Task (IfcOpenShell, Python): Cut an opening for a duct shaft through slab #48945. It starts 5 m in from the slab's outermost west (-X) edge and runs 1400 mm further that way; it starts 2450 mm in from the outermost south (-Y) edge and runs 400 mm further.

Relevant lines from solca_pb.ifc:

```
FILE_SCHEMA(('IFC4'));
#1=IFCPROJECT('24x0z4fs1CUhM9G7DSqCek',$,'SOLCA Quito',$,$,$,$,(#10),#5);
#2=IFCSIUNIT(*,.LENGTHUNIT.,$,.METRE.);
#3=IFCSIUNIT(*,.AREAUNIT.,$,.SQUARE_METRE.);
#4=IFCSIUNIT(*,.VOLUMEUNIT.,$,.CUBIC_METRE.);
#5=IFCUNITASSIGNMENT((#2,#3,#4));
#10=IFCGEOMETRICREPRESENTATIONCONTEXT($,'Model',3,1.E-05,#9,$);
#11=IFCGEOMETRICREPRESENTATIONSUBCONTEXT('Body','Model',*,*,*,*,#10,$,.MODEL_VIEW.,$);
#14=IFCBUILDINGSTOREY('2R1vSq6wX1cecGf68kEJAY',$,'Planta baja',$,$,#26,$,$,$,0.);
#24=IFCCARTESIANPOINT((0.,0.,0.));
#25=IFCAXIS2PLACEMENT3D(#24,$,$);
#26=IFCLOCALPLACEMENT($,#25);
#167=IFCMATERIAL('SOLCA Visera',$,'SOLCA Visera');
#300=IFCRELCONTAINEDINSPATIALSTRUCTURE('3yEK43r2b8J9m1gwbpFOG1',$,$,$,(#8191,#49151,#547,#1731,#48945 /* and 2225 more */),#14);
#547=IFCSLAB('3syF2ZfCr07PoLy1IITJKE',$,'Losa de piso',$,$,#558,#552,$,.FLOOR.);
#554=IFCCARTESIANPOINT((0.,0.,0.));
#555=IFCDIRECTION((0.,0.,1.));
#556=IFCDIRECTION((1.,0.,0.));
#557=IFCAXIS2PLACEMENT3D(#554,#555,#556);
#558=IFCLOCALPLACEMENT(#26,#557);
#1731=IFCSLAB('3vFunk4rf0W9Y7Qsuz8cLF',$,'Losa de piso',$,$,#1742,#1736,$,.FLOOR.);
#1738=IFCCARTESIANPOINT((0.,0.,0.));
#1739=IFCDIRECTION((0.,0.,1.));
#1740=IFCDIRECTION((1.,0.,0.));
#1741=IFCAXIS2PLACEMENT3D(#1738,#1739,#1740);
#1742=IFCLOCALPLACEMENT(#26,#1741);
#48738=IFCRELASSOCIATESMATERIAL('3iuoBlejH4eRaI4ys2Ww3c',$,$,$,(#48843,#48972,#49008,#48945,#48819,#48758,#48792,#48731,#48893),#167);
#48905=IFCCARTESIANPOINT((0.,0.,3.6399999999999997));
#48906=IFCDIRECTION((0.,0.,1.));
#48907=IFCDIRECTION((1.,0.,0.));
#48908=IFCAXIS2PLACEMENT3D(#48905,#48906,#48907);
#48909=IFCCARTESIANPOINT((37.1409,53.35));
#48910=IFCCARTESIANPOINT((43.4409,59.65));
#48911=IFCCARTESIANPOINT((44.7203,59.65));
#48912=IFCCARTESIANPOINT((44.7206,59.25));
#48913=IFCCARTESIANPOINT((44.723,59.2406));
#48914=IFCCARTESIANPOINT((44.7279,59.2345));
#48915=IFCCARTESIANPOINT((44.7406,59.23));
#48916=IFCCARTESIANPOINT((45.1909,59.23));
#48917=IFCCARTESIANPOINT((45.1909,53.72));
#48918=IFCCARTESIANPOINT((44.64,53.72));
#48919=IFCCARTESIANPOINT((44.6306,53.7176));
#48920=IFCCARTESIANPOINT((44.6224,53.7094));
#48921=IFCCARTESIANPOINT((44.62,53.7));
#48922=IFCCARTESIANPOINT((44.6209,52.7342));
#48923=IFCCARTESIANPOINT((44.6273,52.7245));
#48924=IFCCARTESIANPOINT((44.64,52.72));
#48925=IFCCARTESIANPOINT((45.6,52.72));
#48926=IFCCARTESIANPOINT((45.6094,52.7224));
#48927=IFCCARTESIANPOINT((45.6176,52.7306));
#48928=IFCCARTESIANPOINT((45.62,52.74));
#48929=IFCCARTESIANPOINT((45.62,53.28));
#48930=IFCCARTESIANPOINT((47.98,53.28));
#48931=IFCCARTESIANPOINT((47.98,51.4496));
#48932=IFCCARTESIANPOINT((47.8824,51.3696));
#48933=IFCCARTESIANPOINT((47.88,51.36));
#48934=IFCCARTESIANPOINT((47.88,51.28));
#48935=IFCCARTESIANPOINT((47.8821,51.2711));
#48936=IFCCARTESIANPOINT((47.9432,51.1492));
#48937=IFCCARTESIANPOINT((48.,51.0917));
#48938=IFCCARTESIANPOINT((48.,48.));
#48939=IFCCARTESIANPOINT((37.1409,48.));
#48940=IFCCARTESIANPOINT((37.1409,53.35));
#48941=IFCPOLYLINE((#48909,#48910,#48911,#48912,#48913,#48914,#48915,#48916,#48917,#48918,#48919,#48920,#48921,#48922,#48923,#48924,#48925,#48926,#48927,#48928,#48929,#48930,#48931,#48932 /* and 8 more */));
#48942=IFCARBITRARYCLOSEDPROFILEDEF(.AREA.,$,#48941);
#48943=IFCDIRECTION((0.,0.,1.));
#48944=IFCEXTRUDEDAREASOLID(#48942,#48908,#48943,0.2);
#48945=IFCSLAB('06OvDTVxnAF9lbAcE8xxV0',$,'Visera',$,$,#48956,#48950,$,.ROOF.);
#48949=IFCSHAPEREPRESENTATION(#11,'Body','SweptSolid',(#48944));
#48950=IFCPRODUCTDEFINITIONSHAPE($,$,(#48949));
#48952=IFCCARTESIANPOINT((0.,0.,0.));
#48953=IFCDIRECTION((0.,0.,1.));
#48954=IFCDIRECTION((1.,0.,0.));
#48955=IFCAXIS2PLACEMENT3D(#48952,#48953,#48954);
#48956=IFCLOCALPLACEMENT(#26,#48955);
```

```python
import numpy as np
import ifcopenshell
import ifcopenshell.api.feature
import ifcopenshell.api.geometry
import ifcopenshell.api.root
import ifcopenshell.geom
import ifcopenshell.util.placement
import ifcopenshell.util.representation
import ifcopenshell.util.shape
import ifcopenshell.util.unit

model = ifcopenshell.open("solca_pb.ifc")
unit_scale = ifcopenshell.util.unit.calculate_unit_scale(model)
settings = ifcopenshell.geom.settings()


def volume(element):
    """Net volume in cubic metres, openings subtracted."""
    shape = ifcopenshell.geom.create_shape(settings, element)
    return ifcopenshell.util.shape.get_volume(shape.geometry)


slab = model.by_guid("06OvDTVxnAF9lbAcE8xxV0")
before = volume(slab)

# Extent in the slab's own axes, in metres. The edges named are its -X and -Y sides.
slab_shape = ifcopenshell.geom.create_shape(settings, slab)
vertices = ifcopenshell.util.shape.get_vertices(slab_shape.geometry)
x_min, y_min, bottom = vertices.min(axis=0)
top = vertices[:, 2].max()

opening = ifcopenshell.api.root.create_entity(model, ifc_class="IfcOpeningElement", name="Duct shaft opening", predefined_type="OPENING")
context = ifcopenshell.util.representation.get_context(model, "Model", "Body", "MODEL_VIEW")
width, depth = 1.4, 0.4
outline = [(0.0, 0.0), (width, 0.0), (width, depth), (0.0, depth), (0.0, 0.0)]
# Overshoot both faces by 50 mm so the cut is clean.
shape = ifcopenshell.api.geometry.add_slab_representation(
    model, context=context, depth=top - bottom + 0.1, polyline=outline
)
ifcopenshell.api.geometry.assign_representation(model, product=opening, representation=shape)

matrix = ifcopenshell.util.placement.get_local_placement(slab.ObjectPlacement)
matrix[:, 3] = matrix @ np.append(np.array([x_min + 5, y_min + 2.45, bottom - 0.05]) / unit_scale, 1.0)
ifcopenshell.api.geometry.edit_object_placement(model, product=opening, matrix=matrix, is_si=False)
ifcopenshell.api.feature.add_feature(model, feature=opening, element=slab)

after = volume(slab)

print(f"slab volume {before:.3f} -> {after:.3f} m3")

model.write("solca_pb_rev.ifc")
```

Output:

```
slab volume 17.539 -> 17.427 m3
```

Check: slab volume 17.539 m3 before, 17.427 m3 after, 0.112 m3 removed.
